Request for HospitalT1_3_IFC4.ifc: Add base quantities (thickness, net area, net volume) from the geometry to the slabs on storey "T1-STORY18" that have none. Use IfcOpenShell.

First a look at what the model holds.

```python
import ifcopenshell
import ifcopenshell.util.element
import ifcopenshell.util.unit

model = ifcopenshell.open("HospitalT1_3_IFC4.ifc")
print(model.schema)
for unit_type in ("LENGTHUNIT", "AREAUNIT", "VOLUMEUNIT"):
    print(unit_type, ifcopenshell.util.unit.calculate_unit_scale(model, unit_type))
storey = next(s for s in model.by_type("IfcBuildingStorey") if s.Name == "T1-STORY18")
slabs = [e for e in ifcopenshell.util.element.get_decomposition(storey) if e.is_a("IfcSlab")]
for e in sorted(slabs, key=lambda e: e.id()):
    print(e.id(), e.is_a(), e.Name, list(ifcopenshell.util.element.get_psets(e, qtos_only=True)), sep=" | ")
```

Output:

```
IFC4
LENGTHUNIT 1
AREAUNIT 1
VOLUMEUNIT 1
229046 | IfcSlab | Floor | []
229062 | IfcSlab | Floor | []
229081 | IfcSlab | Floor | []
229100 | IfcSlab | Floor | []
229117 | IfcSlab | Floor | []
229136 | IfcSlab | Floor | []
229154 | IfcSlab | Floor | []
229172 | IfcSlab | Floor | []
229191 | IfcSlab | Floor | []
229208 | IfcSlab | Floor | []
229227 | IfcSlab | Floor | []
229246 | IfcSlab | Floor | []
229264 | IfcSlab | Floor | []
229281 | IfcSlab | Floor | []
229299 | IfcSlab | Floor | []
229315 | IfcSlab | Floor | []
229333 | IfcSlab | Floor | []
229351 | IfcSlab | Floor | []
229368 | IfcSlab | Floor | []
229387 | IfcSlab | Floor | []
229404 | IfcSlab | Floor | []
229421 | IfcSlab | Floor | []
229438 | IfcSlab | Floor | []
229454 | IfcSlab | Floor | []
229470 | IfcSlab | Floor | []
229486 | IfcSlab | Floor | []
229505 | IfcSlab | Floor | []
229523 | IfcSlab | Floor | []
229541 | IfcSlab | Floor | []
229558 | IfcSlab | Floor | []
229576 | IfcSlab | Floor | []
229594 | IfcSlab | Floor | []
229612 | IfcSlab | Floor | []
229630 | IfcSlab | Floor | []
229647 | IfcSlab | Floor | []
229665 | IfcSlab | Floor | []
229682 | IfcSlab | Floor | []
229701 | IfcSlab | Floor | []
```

```python
import ifcopenshell
import ifcopenshell.api.pset
import ifcopenshell.geom
import ifcopenshell.util.element
import ifcopenshell.util.shape
import ifcopenshell.util.unit

model = ifcopenshell.open("HospitalT1_3_IFC4.ifc")
unit_scale = ifcopenshell.util.unit.calculate_unit_scale(model)
area_scale = ifcopenshell.util.unit.calculate_unit_scale(model, "AREAUNIT")
volume_scale = ifcopenshell.util.unit.calculate_unit_scale(model, "VOLUMEUNIT")
settings = ifcopenshell.geom.settings()

storey = next(s for s in model.by_type("IfcBuildingStorey") if s.Name == "T1-STORY18")
slabs = [e for e in ifcopenshell.util.element.get_decomposition(storey) if e.is_a("IfcSlab")]

for e in sorted(slabs, key=lambda e: e.id()):
    if ifcopenshell.util.element.get_psets(e, qtos_only=True, should_inherit=False):
        continue
    # Geometry comes back in metres, in the element's own axes.
    shape = ifcopenshell.geom.create_shape(settings, e)
    values = {
        "Width": ifcopenshell.util.shape.get_z(shape.geometry) / unit_scale,
        "NetArea": ifcopenshell.util.shape.get_footprint_area(shape.geometry) / area_scale,
        "NetVolume": ifcopenshell.util.shape.get_volume(shape.geometry) / volume_scale,
    }
    qto = ifcopenshell.api.pset.add_qto(model, product=e, name="Qto_SlabBaseQuantities")
    ifcopenshell.api.pset.edit_qto(model, qto=qto, properties=values)
    print(e.id(), {k: round(v, 3) for k, v in values.items()})

model.write("HospitalT1_3_IFC4_edited.ifc")
```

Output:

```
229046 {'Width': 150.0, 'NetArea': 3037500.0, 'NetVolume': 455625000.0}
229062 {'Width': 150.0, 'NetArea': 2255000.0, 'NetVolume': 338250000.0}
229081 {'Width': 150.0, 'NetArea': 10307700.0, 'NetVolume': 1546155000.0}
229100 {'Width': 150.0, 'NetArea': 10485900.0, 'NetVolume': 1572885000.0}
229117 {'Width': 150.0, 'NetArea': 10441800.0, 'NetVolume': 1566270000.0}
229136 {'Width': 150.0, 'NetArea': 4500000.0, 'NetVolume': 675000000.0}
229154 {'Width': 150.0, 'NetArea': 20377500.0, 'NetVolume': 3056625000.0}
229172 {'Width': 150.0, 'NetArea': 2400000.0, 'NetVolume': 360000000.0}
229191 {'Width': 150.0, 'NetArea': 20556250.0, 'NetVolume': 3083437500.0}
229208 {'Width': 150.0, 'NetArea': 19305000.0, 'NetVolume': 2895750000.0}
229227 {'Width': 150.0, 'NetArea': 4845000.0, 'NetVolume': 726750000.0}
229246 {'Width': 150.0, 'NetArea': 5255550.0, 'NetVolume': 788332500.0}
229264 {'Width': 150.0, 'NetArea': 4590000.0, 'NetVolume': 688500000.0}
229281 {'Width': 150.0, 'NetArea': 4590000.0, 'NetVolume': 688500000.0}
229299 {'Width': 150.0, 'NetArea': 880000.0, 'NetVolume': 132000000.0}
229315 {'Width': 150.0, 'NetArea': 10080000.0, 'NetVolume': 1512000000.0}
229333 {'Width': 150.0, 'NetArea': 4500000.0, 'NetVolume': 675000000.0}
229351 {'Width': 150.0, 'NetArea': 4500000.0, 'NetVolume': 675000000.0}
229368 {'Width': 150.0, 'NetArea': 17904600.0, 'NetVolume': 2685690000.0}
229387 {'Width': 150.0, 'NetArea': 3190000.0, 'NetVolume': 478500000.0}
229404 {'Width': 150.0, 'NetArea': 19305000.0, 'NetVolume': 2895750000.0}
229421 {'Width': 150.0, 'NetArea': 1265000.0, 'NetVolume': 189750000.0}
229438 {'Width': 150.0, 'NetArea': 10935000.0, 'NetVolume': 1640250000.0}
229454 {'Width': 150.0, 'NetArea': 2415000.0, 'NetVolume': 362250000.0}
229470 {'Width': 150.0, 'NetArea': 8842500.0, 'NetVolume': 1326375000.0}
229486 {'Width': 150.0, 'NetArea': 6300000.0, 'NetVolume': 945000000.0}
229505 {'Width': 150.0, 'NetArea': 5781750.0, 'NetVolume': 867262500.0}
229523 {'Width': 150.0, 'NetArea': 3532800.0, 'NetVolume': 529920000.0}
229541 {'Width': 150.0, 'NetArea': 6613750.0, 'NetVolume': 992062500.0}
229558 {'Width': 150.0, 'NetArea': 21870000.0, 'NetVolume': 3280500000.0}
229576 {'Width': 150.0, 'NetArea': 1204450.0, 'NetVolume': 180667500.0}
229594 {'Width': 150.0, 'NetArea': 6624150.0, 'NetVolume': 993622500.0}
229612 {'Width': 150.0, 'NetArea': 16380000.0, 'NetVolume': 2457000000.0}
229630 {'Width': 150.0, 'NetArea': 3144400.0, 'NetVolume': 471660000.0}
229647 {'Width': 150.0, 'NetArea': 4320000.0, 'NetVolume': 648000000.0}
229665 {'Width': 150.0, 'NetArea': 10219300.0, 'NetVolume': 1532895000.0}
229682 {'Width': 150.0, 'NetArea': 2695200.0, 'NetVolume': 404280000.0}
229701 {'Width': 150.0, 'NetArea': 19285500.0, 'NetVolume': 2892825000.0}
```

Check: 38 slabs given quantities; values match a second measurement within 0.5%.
